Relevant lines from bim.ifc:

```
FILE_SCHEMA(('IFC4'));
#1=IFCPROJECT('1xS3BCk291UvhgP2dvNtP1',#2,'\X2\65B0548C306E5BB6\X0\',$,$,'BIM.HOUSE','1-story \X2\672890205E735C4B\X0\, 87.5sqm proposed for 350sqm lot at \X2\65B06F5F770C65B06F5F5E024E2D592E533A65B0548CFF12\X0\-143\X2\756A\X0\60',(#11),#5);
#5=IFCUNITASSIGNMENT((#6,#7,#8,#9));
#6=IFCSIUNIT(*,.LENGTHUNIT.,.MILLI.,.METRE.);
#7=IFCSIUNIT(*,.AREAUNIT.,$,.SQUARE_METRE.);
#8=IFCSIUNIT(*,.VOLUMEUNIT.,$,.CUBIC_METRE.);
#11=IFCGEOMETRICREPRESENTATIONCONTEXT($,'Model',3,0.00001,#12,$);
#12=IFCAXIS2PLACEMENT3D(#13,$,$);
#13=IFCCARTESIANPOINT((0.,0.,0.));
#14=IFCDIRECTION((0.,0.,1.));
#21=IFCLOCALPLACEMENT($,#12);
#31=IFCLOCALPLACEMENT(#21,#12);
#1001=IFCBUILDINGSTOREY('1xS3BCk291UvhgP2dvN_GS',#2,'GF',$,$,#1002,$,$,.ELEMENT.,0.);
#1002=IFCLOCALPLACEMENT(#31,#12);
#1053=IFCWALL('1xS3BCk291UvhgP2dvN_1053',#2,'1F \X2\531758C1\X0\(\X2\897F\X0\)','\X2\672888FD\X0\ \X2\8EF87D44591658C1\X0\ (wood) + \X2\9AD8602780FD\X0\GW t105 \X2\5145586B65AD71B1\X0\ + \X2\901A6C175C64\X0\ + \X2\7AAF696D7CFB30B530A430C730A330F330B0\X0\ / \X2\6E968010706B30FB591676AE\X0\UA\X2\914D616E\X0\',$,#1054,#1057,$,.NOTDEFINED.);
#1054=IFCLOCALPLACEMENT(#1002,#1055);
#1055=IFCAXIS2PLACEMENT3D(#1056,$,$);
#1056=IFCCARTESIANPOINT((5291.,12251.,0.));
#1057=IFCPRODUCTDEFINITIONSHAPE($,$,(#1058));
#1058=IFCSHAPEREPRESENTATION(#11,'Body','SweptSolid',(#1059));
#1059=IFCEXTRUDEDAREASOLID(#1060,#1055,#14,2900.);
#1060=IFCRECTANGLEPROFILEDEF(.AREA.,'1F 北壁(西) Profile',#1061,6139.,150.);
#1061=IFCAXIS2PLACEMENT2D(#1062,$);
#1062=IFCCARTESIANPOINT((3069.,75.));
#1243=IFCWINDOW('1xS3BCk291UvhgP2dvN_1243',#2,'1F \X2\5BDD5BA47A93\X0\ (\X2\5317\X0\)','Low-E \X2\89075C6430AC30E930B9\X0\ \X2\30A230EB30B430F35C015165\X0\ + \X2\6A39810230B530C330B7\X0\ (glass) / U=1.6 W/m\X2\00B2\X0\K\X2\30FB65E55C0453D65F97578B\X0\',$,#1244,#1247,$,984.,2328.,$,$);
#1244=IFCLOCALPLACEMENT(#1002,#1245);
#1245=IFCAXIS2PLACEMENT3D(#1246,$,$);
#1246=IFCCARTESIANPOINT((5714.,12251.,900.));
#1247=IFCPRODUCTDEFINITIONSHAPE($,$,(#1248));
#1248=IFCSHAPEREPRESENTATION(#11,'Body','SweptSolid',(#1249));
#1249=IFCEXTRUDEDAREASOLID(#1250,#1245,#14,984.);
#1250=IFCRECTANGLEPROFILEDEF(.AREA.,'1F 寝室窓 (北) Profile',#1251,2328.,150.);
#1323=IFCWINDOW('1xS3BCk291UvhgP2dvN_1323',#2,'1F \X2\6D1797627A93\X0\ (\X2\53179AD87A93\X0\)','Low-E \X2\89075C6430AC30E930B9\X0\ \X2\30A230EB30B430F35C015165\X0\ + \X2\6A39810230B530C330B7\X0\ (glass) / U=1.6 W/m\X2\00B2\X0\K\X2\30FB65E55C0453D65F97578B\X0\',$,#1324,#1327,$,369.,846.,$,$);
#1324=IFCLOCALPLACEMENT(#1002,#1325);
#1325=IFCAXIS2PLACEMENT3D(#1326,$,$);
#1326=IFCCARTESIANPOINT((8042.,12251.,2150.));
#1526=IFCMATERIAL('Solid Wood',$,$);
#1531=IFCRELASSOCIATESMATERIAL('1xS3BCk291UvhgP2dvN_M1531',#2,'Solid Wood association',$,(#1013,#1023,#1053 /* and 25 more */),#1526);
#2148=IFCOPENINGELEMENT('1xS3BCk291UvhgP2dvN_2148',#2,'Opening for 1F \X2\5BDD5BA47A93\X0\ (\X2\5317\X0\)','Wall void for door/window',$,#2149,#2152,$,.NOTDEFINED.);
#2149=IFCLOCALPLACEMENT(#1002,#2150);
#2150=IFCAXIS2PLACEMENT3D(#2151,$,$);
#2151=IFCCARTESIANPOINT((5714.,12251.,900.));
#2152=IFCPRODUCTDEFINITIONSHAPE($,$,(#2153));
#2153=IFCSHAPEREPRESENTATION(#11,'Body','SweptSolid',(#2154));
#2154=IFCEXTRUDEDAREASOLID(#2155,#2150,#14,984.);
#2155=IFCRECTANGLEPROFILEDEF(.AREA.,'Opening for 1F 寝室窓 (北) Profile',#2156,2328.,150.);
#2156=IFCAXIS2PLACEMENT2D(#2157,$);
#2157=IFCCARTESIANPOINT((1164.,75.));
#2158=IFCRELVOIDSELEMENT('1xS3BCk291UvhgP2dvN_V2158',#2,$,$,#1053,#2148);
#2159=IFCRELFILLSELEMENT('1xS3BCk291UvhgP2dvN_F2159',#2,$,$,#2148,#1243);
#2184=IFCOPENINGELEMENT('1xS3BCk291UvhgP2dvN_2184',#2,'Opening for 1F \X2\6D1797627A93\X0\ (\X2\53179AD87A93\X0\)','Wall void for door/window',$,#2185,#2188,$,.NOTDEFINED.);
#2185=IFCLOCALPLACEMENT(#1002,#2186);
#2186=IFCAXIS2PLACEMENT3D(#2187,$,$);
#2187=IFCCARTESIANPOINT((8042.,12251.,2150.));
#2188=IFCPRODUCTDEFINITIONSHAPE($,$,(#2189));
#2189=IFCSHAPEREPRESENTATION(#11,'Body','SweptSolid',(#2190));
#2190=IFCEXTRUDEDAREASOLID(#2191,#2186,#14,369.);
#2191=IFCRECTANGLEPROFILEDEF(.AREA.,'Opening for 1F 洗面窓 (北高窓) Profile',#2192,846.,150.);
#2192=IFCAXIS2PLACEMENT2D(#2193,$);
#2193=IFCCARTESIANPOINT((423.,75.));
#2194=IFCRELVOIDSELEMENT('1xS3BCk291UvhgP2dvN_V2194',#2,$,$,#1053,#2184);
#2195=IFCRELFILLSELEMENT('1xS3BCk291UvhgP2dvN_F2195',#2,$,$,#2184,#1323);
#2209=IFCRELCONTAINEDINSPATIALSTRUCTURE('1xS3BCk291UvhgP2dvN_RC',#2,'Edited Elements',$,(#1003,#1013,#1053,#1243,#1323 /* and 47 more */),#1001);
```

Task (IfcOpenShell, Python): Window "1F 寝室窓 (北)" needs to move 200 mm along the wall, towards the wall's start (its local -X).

```python
import ifcopenshell
import ifcopenshell.api.geometry
import ifcopenshell.util.placement
import ifcopenshell.util.unit

model = ifcopenshell.open("bim.ifc")
unit_scale = ifcopenshell.util.unit.calculate_unit_scale(model)

window = model.by_id(1243)
opening = window.FillsVoids[0].RelatingOpeningElement
wall = opening.VoidsElements[0].RelatingBuildingElement

wall_matrix = ifcopenshell.util.placement.get_local_placement(wall.ObjectPlacement)
shift = wall_matrix[:3, 0] * -0.2 / unit_scale
before = ifcopenshell.util.placement.get_local_placement(window.ObjectPlacement)[:3, 3].copy()

# The window is not placed relative to its opening, so move both.
for product in (opening, window):
    matrix = ifcopenshell.util.placement.get_local_placement(product.ObjectPlacement)
    matrix[:3, 3] += shift
    ifcopenshell.api.geometry.edit_object_placement(model, product=product, matrix=matrix, is_si=False)

after = ifcopenshell.util.placement.get_local_placement(window.ObjectPlacement)[:3, 3]
print("window moved by", (after - before).round(3) + 0.0)

model.write("bim_edited.ifc")
```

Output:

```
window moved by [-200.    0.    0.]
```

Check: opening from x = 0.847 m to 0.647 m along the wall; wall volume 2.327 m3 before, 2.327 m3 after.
